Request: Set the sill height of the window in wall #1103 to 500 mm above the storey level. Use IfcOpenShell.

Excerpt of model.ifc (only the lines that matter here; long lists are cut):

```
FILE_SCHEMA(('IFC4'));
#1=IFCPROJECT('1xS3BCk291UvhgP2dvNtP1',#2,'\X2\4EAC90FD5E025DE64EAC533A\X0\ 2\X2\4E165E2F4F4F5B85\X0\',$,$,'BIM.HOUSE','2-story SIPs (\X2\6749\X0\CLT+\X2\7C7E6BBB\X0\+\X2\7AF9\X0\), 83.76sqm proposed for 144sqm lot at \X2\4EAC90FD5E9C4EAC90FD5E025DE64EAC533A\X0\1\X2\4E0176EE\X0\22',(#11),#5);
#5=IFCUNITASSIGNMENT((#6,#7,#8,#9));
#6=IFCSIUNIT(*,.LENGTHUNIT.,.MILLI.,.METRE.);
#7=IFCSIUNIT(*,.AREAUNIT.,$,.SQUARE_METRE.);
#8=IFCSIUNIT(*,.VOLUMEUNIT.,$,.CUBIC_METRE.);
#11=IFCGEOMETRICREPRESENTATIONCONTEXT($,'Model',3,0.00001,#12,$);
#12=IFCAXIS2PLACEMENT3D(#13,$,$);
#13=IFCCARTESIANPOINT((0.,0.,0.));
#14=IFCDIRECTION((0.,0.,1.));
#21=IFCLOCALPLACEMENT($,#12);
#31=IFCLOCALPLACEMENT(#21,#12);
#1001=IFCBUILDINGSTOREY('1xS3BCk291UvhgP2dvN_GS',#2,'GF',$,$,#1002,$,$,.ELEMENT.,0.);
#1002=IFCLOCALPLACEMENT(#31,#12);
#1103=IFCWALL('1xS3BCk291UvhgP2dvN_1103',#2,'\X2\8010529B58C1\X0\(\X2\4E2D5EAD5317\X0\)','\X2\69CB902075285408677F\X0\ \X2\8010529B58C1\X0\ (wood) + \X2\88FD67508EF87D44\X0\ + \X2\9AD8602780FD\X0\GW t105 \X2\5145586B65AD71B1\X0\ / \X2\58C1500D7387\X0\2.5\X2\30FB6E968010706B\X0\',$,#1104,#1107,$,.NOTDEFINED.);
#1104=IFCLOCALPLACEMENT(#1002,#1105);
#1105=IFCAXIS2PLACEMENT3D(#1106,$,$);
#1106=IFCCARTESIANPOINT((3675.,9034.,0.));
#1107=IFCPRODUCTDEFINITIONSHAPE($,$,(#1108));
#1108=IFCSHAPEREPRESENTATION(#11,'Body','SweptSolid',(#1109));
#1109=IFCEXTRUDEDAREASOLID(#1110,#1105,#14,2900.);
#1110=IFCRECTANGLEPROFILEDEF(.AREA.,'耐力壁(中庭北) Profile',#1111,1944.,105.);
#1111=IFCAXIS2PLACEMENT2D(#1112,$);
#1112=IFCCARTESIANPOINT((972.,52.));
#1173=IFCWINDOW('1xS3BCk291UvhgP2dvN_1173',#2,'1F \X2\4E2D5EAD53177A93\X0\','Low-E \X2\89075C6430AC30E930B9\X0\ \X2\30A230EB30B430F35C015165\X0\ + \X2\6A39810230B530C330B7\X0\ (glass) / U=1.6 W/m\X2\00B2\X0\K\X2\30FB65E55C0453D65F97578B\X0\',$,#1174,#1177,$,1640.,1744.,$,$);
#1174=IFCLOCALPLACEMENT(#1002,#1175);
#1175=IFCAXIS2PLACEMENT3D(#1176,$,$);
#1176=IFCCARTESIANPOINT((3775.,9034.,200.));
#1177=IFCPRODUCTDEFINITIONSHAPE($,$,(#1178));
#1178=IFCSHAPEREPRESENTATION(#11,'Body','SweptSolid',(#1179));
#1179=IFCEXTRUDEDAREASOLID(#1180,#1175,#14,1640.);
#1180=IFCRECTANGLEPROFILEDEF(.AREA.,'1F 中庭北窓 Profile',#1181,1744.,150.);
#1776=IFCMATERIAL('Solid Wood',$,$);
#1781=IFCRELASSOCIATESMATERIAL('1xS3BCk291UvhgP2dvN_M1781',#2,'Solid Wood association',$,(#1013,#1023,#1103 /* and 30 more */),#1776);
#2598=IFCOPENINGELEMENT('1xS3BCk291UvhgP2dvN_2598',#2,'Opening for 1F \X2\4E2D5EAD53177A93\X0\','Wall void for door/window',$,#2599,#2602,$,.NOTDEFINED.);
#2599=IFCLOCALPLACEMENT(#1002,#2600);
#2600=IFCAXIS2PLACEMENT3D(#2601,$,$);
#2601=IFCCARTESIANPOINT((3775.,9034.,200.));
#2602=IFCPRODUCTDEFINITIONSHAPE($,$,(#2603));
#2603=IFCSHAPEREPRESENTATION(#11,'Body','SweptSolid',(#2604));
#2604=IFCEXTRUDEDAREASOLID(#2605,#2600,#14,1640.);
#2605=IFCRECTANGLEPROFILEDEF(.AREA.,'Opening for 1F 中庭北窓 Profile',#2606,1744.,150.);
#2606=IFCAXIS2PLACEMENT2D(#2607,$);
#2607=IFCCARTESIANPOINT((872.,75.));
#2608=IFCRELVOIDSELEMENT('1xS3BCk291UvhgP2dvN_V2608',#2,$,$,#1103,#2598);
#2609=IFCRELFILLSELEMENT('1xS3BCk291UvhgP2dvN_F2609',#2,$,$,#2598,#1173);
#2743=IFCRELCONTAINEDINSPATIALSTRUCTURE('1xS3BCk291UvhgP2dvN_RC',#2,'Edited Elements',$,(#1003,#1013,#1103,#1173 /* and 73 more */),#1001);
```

```python
import numpy as np
import ifcopenshell
import ifcopenshell.api.geometry
import ifcopenshell.geom
import ifcopenshell.util.element
import ifcopenshell.util.placement
import ifcopenshell.util.shape
import ifcopenshell.util.unit

model = ifcopenshell.open("model.ifc")
unit_scale = ifcopenshell.util.unit.calculate_unit_scale(model)

window = model.by_guid("1xS3BCk291UvhgP2dvN_1173")
opening = window.FillsVoids[0].RelatingOpeningElement
storey = ifcopenshell.util.element.get_container(window, ifc_class="IfcBuildingStorey")
level = ifcopenshell.util.placement.get_local_placement(storey.ObjectPlacement)[2, 3]

# The opening's origin need not be at the sill, so measure its lowest point.
shape = ifcopenshell.geom.create_shape(ifcopenshell.geom.settings(), opening)
bottom = ifcopenshell.util.shape.get_shape_bottom_elevation(shape, shape.geometry) / unit_scale
dz = level + 0.5 / unit_scale - bottom

shift = np.array([0.0, 0.0, dz])
# The window is not placed relative to its opening, so move both.
for product in (opening, window):
    matrix = ifcopenshell.util.placement.get_local_placement(product.ObjectPlacement)
    matrix[:3, 3] += shift
    ifcopenshell.api.geometry.edit_object_placement(model, product=product, matrix=matrix, is_si=False)

print(f"moved by {dz * unit_scale:+.3f} m")

model.write("model_updated.ifc")
```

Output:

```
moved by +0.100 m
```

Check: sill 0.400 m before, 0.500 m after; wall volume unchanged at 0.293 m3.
